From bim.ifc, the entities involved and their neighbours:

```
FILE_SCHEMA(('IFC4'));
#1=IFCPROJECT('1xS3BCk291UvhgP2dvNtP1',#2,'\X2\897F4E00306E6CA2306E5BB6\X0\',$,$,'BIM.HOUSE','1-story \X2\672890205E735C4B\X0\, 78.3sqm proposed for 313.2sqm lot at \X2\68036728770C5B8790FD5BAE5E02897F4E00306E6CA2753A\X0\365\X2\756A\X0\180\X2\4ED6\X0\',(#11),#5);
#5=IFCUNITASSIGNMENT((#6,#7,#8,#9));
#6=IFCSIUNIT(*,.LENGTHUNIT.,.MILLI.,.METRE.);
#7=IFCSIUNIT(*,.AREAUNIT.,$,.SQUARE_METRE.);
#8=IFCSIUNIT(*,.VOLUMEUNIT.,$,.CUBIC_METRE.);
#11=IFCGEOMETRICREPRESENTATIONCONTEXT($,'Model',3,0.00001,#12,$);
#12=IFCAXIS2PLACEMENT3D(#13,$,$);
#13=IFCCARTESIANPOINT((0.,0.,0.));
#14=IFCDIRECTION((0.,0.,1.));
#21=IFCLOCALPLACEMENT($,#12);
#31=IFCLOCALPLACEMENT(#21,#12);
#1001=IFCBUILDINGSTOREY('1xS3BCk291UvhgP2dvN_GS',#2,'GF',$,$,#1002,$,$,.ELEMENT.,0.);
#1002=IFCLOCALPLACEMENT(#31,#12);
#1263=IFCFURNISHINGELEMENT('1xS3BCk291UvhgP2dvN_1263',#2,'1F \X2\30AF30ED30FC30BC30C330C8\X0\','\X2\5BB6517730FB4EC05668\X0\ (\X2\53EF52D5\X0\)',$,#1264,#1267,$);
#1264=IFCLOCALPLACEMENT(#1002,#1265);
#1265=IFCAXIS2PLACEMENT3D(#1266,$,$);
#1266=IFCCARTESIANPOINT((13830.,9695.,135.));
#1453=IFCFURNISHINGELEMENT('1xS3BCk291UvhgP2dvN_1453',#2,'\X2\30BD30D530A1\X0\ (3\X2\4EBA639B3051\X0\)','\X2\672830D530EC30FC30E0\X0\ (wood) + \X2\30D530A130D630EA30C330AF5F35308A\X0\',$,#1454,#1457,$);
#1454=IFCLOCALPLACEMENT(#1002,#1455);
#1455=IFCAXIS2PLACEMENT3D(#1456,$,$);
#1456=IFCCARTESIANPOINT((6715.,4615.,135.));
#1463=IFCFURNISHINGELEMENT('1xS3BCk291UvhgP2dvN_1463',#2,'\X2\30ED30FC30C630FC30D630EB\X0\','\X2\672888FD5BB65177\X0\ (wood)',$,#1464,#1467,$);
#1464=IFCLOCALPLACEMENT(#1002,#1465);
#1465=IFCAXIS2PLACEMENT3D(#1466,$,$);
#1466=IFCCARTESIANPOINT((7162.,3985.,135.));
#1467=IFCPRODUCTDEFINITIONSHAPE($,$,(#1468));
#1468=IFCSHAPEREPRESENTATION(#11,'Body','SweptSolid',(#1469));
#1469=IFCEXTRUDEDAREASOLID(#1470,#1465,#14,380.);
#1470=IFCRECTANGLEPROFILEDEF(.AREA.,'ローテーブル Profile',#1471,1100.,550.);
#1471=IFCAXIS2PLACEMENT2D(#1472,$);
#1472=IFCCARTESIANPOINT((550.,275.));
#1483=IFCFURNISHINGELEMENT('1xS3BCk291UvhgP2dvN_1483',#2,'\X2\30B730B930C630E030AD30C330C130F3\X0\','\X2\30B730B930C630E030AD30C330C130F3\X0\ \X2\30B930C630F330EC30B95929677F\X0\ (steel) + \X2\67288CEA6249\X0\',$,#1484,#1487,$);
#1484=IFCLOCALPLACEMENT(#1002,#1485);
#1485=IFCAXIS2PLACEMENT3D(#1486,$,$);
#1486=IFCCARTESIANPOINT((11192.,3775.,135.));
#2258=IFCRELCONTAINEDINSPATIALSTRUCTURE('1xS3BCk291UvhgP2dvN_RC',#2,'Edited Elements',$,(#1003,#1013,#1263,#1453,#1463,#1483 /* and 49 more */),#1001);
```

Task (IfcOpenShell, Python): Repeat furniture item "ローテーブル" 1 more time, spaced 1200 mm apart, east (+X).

```python
import numpy as np
import ifcopenshell
import ifcopenshell.api.geometry
import ifcopenshell.api.root
import ifcopenshell.util.element
import ifcopenshell.util.placement

model = ifcopenshell.open("bim.ifc")


def reuse_history(source, copy):
    """copy_class also copies each property set's owner history, people and application; keep the originals."""
    for rel in copy.IsDefinedBy:
        if rel.is_a("IfcRelDefinesByProperties") and (history := rel.RelatingPropertyDefinition.OwnerHistory):
            rel.RelatingPropertyDefinition.OwnerHistory = source.OwnerHistory
            ifcopenshell.util.element.remove_deep2(model, history)


source = model.by_guid("1xS3BCk291UvhgP2dvN_1463")
base = ifcopenshell.util.placement.get_local_placement(source.ObjectPlacement)
step = np.array([1.0, 0.0, 0.0]) * 1200.0

for i in range(1, 2):
    copy = ifcopenshell.api.root.copy_class(model, product=source)
    copy.Representation = ifcopenshell.util.element.copy_deep(
        model, source.Representation, exclude=["IfcGeometricRepresentationContext", "IfcRepresentationMap"]
    )
    reuse_history(source, copy)
    matrix = base.copy()
    matrix[:3, 3] += i * step
    print("added at", matrix[:3, 3].round(3) + 0.0)
    ifcopenshell.api.geometry.edit_object_placement(model, product=copy, matrix=matrix, is_si=False)

model.write("bim-out.ifc")
```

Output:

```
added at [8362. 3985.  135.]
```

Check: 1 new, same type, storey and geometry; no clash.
